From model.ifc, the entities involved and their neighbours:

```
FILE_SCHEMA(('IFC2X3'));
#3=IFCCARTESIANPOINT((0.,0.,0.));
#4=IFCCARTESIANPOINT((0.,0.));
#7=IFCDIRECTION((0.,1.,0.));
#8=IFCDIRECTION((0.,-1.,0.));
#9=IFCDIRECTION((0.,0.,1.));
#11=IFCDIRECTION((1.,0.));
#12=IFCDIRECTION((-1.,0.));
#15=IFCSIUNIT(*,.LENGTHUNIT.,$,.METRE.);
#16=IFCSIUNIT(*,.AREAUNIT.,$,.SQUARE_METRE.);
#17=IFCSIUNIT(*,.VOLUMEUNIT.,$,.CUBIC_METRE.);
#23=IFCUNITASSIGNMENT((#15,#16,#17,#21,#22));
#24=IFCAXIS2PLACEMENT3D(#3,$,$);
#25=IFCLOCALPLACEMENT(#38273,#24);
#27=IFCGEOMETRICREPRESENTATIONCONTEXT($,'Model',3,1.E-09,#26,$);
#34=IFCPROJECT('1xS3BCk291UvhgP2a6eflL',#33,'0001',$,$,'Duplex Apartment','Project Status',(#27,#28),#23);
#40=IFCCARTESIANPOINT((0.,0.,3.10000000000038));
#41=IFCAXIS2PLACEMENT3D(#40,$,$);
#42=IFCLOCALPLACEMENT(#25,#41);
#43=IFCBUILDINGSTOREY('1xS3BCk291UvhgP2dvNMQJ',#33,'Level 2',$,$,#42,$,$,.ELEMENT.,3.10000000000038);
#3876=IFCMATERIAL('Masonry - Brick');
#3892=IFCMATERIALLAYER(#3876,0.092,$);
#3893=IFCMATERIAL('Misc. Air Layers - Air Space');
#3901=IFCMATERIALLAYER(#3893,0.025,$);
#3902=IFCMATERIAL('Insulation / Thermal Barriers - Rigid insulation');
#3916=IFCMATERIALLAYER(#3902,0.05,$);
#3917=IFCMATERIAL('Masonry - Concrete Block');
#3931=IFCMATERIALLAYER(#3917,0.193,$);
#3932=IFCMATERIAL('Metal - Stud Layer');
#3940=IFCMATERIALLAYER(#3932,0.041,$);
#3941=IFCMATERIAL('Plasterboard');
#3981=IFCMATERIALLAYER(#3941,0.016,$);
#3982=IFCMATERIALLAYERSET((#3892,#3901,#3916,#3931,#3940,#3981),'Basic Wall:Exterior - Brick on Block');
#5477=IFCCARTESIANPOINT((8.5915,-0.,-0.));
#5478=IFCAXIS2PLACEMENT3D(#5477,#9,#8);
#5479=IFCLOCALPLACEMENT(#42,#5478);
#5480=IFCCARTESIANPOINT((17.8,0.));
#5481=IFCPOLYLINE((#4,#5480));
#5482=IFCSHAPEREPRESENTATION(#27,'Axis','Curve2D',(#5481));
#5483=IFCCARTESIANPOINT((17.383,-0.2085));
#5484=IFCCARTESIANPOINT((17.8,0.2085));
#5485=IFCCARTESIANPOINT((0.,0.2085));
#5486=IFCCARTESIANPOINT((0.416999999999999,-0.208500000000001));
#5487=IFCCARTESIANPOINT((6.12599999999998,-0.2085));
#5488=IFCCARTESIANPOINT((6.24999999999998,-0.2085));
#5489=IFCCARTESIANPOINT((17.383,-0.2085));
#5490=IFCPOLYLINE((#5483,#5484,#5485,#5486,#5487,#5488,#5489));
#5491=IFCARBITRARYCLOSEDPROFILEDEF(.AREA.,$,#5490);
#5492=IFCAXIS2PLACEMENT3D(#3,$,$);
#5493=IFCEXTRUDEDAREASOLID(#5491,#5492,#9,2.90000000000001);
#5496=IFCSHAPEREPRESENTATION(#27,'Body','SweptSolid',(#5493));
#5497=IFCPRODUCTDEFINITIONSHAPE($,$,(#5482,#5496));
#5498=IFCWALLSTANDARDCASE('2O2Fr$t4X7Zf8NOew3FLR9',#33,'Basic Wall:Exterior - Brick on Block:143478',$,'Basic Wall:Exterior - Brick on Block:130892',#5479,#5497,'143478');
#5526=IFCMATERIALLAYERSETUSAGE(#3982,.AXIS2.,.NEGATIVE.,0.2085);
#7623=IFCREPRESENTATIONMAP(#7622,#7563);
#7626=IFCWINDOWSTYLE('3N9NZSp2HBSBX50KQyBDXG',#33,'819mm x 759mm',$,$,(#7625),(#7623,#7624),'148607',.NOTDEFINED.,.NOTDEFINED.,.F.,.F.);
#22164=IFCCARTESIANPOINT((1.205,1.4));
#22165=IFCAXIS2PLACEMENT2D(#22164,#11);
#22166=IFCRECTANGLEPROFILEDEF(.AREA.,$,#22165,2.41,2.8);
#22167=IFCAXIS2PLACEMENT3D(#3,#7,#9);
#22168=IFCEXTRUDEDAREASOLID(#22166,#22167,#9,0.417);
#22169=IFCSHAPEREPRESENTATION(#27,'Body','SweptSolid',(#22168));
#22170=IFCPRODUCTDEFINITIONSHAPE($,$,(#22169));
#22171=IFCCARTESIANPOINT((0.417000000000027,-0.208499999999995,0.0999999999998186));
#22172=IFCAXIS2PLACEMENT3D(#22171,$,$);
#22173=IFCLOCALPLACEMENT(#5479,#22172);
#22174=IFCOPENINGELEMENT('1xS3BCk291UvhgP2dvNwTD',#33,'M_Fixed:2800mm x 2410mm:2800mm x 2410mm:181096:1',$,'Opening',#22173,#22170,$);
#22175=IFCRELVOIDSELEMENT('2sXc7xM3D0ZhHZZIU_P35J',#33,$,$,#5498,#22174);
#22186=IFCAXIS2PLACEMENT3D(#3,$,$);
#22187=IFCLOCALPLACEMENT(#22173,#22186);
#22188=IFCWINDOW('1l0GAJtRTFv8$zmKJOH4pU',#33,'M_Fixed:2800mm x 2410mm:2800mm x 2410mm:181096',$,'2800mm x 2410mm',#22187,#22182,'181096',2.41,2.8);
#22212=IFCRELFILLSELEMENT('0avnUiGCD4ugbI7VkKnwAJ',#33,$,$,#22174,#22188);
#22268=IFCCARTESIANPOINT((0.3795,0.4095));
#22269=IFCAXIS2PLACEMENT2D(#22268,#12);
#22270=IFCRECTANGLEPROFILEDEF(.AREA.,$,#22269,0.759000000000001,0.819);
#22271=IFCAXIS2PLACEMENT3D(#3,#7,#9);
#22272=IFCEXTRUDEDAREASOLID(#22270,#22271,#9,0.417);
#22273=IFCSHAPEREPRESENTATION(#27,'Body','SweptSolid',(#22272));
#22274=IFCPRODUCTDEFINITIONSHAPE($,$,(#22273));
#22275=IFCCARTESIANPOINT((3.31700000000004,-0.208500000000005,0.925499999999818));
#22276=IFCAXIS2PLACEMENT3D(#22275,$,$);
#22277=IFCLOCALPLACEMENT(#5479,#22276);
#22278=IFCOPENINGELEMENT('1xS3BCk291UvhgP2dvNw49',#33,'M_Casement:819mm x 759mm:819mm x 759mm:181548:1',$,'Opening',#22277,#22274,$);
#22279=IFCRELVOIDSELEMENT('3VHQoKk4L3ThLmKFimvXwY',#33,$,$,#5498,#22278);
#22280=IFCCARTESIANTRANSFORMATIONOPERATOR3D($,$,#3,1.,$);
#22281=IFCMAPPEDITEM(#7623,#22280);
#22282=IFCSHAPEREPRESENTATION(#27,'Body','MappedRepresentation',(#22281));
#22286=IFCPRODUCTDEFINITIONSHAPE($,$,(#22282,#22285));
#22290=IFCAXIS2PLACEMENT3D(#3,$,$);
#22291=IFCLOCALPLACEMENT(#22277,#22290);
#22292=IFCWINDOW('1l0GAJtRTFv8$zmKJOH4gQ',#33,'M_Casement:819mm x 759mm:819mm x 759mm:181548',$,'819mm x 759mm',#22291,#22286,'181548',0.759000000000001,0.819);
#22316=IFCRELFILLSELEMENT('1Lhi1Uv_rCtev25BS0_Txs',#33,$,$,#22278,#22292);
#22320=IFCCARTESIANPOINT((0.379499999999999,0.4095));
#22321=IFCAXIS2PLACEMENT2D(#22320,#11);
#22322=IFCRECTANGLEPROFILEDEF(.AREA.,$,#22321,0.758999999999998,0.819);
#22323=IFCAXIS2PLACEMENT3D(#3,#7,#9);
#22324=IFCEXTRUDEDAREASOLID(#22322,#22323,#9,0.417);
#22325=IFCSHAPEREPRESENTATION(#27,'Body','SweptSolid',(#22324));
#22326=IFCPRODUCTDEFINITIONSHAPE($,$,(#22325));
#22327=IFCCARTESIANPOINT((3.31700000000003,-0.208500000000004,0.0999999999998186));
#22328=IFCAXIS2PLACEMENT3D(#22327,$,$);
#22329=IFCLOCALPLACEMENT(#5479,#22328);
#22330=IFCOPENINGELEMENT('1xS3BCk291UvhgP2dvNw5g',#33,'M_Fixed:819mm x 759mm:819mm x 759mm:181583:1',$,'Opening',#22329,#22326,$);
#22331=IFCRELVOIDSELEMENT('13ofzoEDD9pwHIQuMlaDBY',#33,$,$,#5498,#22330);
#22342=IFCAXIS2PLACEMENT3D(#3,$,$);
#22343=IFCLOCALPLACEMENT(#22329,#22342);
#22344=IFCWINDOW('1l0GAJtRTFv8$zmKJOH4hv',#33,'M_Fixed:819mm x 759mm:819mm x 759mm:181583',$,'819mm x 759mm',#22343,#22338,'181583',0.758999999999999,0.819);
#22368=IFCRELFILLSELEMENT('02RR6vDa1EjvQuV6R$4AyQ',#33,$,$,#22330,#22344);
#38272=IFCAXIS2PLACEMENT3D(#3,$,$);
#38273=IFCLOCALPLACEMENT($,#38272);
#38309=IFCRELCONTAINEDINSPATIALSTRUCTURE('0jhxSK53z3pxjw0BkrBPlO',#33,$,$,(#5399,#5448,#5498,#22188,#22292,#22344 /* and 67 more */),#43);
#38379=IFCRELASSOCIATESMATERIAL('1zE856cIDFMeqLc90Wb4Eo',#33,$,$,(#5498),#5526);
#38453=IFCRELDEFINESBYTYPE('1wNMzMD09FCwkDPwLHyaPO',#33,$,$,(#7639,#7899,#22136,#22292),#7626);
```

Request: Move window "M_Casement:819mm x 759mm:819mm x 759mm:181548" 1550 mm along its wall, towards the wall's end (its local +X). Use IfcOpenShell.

```python
import ifcopenshell
import ifcopenshell.api.geometry
import ifcopenshell.util.placement
import ifcopenshell.util.unit

model = ifcopenshell.open("model.ifc")
unit_scale = ifcopenshell.util.unit.calculate_unit_scale(model)

window = model.by_guid("1l0GAJtRTFv8$zmKJOH4gQ")
opening = window.FillsVoids[0].RelatingOpeningElement
wall = opening.VoidsElements[0].RelatingBuildingElement

wall_matrix = ifcopenshell.util.placement.get_local_placement(wall.ObjectPlacement)
shift = wall_matrix[:3, 0] * 1.55 / unit_scale
before = ifcopenshell.util.placement.get_local_placement(window.ObjectPlacement)[:3, 3].copy()

# The window is placed relative to its opening, so it follows when the opening moves.
matrix = ifcopenshell.util.placement.get_local_placement(opening.ObjectPlacement)
matrix[:3, 3] += shift
ifcopenshell.api.geometry.edit_object_placement(
    model, product=opening, matrix=matrix, is_si=False, should_transform_children=True
)

after = ifcopenshell.util.placement.get_local_placement(window.ObjectPlacement)[:3, 3]
print("window moved by", (after - before).round(3) + 0.0)

model.write("model-out.ifc")
```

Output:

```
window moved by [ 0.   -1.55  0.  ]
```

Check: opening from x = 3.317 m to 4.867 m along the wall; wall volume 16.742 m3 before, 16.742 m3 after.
